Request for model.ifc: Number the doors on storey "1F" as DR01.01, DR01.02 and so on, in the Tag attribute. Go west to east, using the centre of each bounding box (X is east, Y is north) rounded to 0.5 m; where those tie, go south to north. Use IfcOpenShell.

First a look at what the model holds.

```python
import ifcopenshell
import ifcopenshell.util.element
import ifcopenshell.util.placement

model = ifcopenshell.open("model.ifc")
print(model.schema)
storey = next(s for s in model.by_type("IfcBuildingStorey") if s.Name == "1F")
doors = [e for e in ifcopenshell.util.element.get_decomposition(storey) if e.is_a("IfcDoor")]
for e in sorted(doors, key=lambda e: e.id()):
    origin = ifcopenshell.util.placement.get_local_placement(e.ObjectPlacement)[:3, 3]
    print(e.id(), e.Tag, e.Name, origin.round(2) + 0.0, sep=" | ")
```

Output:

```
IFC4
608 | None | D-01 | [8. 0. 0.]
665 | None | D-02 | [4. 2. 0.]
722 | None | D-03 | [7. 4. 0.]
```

```python
import ifcopenshell
import ifcopenshell.geom
import ifcopenshell.util.element
import ifcopenshell.util.shape

model = ifcopenshell.open("model.ifc")
settings = ifcopenshell.geom.settings()
settings.set("use-world-coords", True)


def centre(element):
    shape = ifcopenshell.geom.create_shape(settings, element)
    return ifcopenshell.util.shape.get_bbox_centroid(shape.geometry)


storey = next(s for s in model.by_type("IfcBuildingStorey") if s.Name == "1F")
doors = [e for e in ifcopenshell.util.element.get_decomposition(storey) if e.is_a("IfcDoor")]

# Insertion points can sit at a corner or the storey origin, so sort by the geometry (in metres).
centres = {e: centre(e) for e in doors}
doors.sort(key=lambda e: (round(centres[e][0] / 0.5), centres[e][1]))

for i, e in enumerate(doors, start=1):
    number = f"DR01.{i:02d}"
    e.Tag = number
    print(e.id(), number)

model.write("model_edited.ifc")
```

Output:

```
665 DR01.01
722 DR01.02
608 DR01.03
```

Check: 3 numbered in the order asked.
